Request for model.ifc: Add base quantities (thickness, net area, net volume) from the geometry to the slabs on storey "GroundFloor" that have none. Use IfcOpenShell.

First a look at what the model holds.

```python
import ifcopenshell
import ifcopenshell.util.element
import ifcopenshell.util.unit

model = ifcopenshell.open("model.ifc")
print(model.schema)
for unit_type in ("LENGTHUNIT", "AREAUNIT", "VOLUMEUNIT"):
    print(unit_type, ifcopenshell.util.unit.calculate_unit_scale(model, unit_type))
storey = next(s for s in model.by_type("IfcBuildingStorey") if s.Name == "GroundFloor")
slabs = [e for e in ifcopenshell.util.element.get_decomposition(storey) if e.is_a("IfcSlab")]
for e in sorted(slabs, key=lambda e: e.id()):
    print(e.id(), e.is_a(), e.Name, list(ifcopenshell.util.element.get_psets(e, qtos_only=True)), sep=" | ")
```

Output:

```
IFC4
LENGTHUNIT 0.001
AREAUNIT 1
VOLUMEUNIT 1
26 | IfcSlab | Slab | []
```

```python
import ifcopenshell
import ifcopenshell.api.pset
import ifcopenshell.geom
import ifcopenshell.util.element
import ifcopenshell.util.shape
import ifcopenshell.util.unit

model = ifcopenshell.open("model.ifc")
unit_scale = ifcopenshell.util.unit.calculate_unit_scale(model)
area_scale = ifcopenshell.util.unit.calculate_unit_scale(model, "AREAUNIT")
volume_scale = ifcopenshell.util.unit.calculate_unit_scale(model, "VOLUMEUNIT")
settings = ifcopenshell.geom.settings()

storey = next(s for s in model.by_type("IfcBuildingStorey") if s.Name == "GroundFloor")
slabs = [e for e in ifcopenshell.util.element.get_decomposition(storey) if e.is_a("IfcSlab")]

for e in sorted(slabs, key=lambda e: e.id()):
    if ifcopenshell.util.element.get_psets(e, qtos_only=True, should_inherit=False):
        continue
    # Geometry comes back in metres, in the element's own axes.
    shape = ifcopenshell.geom.create_shape(settings, e)
    values = {
        "Width": ifcopenshell.util.shape.get_z(shape.geometry) / unit_scale,
        "NetArea": ifcopenshell.util.shape.get_footprint_area(shape.geometry) / area_scale,
        "NetVolume": ifcopenshell.util.shape.get_volume(shape.geometry) / volume_scale,
    }
    qto = ifcopenshell.api.pset.add_qto(model, product=e, name="Qto_SlabBaseQuantities")
    ifcopenshell.api.pset.edit_qto(model, qto=qto, properties=values)
    print(e.id(), {k: round(v, 3) for k, v in values.items()})

model.write("model_edited.ifc")
```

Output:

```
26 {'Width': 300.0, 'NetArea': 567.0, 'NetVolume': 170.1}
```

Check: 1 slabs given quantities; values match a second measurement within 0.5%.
